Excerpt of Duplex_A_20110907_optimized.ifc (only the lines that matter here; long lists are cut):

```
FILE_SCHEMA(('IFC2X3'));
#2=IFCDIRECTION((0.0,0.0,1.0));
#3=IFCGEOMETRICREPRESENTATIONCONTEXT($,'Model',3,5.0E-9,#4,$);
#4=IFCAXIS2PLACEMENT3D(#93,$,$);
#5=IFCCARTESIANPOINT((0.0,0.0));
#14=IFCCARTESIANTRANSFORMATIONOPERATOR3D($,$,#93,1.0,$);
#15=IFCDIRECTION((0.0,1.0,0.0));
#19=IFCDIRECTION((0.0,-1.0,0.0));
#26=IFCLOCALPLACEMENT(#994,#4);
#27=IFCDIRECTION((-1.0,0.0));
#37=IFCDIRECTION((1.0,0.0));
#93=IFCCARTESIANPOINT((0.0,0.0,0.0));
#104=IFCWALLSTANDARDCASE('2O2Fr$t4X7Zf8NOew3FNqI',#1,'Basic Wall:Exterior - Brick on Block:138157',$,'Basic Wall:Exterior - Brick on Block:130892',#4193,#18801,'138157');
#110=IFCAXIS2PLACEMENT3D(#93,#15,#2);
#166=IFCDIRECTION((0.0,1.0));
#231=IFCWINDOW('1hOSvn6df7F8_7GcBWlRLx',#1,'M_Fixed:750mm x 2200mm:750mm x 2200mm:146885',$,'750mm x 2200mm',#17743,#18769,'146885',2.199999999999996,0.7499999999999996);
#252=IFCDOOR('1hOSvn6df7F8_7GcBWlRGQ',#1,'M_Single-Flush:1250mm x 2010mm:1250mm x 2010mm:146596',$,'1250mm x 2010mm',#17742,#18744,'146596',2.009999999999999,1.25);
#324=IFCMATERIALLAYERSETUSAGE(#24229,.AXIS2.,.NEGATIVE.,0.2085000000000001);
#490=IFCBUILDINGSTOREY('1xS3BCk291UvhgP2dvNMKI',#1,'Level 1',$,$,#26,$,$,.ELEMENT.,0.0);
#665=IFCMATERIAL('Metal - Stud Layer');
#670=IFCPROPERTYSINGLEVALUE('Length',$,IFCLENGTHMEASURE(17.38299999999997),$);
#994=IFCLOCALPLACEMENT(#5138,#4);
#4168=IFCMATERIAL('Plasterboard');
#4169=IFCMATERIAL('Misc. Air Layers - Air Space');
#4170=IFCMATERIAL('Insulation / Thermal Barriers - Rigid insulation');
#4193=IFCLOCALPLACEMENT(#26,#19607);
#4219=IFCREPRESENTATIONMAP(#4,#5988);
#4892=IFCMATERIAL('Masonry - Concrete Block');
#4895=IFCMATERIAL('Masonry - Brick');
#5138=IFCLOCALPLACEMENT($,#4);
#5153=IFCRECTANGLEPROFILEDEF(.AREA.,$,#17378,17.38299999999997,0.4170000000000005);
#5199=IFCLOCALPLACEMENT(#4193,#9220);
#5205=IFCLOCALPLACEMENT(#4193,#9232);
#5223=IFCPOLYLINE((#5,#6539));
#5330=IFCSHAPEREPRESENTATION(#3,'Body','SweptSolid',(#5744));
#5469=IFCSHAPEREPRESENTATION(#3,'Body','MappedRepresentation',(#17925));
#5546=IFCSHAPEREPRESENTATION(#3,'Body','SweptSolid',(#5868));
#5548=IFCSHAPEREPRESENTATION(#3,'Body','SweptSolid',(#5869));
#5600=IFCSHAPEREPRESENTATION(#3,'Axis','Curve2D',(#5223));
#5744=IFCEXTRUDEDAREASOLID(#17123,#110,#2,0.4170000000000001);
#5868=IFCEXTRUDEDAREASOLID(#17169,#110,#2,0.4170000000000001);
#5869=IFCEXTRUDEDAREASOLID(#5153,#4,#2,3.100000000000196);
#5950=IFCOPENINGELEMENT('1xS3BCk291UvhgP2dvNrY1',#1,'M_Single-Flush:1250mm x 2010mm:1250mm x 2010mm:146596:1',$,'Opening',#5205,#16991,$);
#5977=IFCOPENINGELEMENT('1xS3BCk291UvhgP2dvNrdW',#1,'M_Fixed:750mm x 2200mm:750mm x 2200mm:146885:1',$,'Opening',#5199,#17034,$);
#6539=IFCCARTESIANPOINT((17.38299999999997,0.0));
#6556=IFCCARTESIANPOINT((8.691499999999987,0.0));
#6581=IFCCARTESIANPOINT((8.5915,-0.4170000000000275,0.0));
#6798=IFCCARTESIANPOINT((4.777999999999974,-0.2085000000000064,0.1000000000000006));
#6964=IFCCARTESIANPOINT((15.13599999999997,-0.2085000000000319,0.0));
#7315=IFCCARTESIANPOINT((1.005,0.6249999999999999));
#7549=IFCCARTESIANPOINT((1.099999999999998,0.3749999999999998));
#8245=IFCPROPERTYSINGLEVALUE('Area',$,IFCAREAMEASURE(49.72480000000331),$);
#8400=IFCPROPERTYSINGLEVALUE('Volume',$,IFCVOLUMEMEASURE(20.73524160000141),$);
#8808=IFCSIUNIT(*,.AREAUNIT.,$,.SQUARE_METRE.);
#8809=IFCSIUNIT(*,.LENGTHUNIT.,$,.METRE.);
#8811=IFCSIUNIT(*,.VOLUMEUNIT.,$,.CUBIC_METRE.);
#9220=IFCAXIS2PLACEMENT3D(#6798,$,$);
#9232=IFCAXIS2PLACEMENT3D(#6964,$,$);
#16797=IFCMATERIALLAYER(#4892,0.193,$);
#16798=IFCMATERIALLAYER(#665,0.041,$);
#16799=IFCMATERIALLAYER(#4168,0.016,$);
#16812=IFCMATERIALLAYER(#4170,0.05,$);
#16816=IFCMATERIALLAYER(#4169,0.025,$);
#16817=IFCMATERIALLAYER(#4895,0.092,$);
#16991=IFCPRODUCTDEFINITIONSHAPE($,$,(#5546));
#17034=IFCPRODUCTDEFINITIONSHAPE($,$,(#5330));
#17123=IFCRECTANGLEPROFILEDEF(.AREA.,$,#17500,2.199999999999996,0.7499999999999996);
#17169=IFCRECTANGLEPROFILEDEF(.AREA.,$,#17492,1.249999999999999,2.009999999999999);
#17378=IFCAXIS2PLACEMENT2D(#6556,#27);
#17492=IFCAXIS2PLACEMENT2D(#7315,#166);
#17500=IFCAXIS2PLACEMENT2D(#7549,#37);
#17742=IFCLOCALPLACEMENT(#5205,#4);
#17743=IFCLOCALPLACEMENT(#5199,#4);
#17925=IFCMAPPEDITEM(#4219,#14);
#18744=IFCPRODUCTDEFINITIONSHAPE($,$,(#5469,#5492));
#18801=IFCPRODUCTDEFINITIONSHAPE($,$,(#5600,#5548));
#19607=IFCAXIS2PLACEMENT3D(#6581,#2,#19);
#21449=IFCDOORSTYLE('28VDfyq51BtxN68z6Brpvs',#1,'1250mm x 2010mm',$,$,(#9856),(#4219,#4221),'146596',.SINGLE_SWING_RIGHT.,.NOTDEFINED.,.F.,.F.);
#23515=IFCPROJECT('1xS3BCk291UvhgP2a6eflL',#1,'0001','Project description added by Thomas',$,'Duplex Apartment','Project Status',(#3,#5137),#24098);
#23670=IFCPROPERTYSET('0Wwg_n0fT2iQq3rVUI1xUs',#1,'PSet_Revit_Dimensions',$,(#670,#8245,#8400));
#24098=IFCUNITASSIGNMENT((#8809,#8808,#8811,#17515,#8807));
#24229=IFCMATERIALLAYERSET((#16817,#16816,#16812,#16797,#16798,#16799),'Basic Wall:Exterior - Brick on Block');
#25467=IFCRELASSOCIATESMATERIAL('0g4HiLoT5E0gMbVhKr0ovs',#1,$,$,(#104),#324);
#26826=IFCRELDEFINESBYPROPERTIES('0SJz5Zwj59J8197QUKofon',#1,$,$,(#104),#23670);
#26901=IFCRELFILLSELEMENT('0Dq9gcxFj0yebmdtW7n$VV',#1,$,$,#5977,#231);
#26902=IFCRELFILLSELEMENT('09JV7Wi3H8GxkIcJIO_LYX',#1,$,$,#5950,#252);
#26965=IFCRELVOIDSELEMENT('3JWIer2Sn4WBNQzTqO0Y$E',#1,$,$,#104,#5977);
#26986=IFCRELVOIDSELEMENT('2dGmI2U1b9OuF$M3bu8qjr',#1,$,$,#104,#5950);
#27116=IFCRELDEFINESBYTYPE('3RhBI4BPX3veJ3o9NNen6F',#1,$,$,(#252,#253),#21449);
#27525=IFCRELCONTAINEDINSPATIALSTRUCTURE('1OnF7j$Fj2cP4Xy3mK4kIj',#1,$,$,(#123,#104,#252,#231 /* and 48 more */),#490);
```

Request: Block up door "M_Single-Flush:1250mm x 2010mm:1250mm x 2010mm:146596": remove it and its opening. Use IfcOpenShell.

```python
import ifcopenshell
import ifcopenshell.api.feature
import ifcopenshell.api.pset
import ifcopenshell.api.root
import ifcopenshell.geom
import ifcopenshell.util.element
import ifcopenshell.util.shape
import ifcopenshell.util.unit

model = ifcopenshell.open("Duplex_A_20110907_optimized.ifc")
area_scale = ifcopenshell.util.unit.calculate_unit_scale(model, "AREAUNIT")
volume_scale = ifcopenshell.util.unit.calculate_unit_scale(model, "VOLUMEUNIT")
settings = ifcopenshell.geom.settings()


def volume(element):
    """Net volume in cubic metres, openings subtracted."""
    shape = ifcopenshell.geom.create_shape(settings, element)
    return ifcopenshell.util.shape.get_volume(shape.geometry)


door = model.by_guid("1hOSvn6df7F8_7GcBWlRGQ")
opening = door.FillsVoids[0].RelatingOpeningElement
wall = opening.VoidsElements[0].RelatingBuildingElement
before = volume(wall)

ifcopenshell.api.root.remove_product(model, product=door)
ifcopenshell.api.feature.remove_feature(model, feature=opening)

after = volume(wall)
thickness = 0.417  # wall thickness in metres

# Update the wall's stored quantities.
pset = model.by_id(ifcopenshell.util.element.get_pset(wall, "PSet_Revit_Dimensions", should_inherit=False)["id"])
ifcopenshell.api.pset.edit_pset(model, pset=pset, properties={
    "Area": model.create_entity("IfcAreaMeasure", after / thickness / area_scale),
    "Volume": model.create_entity("IfcVolumeMeasure", after / volume_scale),
})

print(f"wall volume {before:.3f} -> {after:.3f} m3")

model.write("Duplex_A_20110907_optimized_updated.ifc")
```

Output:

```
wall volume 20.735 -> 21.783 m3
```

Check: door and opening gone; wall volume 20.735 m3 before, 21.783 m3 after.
